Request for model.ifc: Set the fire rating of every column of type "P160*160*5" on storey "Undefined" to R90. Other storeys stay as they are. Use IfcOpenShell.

First a look at what the model holds.

```python
import ifcopenshell
import ifcopenshell.util.element

model = ifcopenshell.open("model.ifc")
print(model.schema)
storey = next(s for s in model.by_type("IfcBuildingStorey") if s.Name == "Undefined")
columns = [e for e in ifcopenshell.util.element.get_decomposition(storey) if e.is_a("IfcColumn")]
seen = {}
for e in columns:
    element_type = ifcopenshell.util.element.get_type(e)
    key = (element_type.Name if element_type != e and element_type else None, ifcopenshell.util.element.get_pset(e, "Pset_ColumnCommon", "FireRating"))
    seen[key] = seen.get(key, 0) + 1
for (name, value), count in sorted(seen.items(), key=str):
    print(count, "x", name, "|", value)
```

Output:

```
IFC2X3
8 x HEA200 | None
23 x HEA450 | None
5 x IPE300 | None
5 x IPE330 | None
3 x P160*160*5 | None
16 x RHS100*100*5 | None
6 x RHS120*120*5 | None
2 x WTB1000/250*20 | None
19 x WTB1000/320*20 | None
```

```python
import ifcopenshell
import ifcopenshell.api.pset
import ifcopenshell.util.element

model = ifcopenshell.open("model.ifc")

storey = next(s for s in model.by_type("IfcBuildingStorey") if s.Name == "Undefined")
columns = [e for e in ifcopenshell.util.element.get_decomposition(storey) if e.is_a("IfcColumn")]

count = 0
for e in columns:
    element_type = ifcopenshell.util.element.get_type(e)
    if element_type in (None, e) or element_type.Name != "P160*160*5":
        continue
    found = ifcopenshell.util.element.get_pset(e, "Pset_ColumnCommon", should_inherit=False)
    if found:
        pset = model.by_id(found["id"])
        if len(ifcopenshell.util.element.get_elements_by_pset(pset)) > 1:
            pset = ifcopenshell.api.pset.unshare_pset(model, products=[e], pset=pset)[0]
    else:
        pset = ifcopenshell.api.pset.add_pset(model, product=e, name="Pset_ColumnCommon")
    ifcopenshell.api.pset.edit_pset(model, pset=pset, properties={"FireRating": "R90"})
    count += 1

print(count, "columns updated")

model.write("model-out.ifc")
```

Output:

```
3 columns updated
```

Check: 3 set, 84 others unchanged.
